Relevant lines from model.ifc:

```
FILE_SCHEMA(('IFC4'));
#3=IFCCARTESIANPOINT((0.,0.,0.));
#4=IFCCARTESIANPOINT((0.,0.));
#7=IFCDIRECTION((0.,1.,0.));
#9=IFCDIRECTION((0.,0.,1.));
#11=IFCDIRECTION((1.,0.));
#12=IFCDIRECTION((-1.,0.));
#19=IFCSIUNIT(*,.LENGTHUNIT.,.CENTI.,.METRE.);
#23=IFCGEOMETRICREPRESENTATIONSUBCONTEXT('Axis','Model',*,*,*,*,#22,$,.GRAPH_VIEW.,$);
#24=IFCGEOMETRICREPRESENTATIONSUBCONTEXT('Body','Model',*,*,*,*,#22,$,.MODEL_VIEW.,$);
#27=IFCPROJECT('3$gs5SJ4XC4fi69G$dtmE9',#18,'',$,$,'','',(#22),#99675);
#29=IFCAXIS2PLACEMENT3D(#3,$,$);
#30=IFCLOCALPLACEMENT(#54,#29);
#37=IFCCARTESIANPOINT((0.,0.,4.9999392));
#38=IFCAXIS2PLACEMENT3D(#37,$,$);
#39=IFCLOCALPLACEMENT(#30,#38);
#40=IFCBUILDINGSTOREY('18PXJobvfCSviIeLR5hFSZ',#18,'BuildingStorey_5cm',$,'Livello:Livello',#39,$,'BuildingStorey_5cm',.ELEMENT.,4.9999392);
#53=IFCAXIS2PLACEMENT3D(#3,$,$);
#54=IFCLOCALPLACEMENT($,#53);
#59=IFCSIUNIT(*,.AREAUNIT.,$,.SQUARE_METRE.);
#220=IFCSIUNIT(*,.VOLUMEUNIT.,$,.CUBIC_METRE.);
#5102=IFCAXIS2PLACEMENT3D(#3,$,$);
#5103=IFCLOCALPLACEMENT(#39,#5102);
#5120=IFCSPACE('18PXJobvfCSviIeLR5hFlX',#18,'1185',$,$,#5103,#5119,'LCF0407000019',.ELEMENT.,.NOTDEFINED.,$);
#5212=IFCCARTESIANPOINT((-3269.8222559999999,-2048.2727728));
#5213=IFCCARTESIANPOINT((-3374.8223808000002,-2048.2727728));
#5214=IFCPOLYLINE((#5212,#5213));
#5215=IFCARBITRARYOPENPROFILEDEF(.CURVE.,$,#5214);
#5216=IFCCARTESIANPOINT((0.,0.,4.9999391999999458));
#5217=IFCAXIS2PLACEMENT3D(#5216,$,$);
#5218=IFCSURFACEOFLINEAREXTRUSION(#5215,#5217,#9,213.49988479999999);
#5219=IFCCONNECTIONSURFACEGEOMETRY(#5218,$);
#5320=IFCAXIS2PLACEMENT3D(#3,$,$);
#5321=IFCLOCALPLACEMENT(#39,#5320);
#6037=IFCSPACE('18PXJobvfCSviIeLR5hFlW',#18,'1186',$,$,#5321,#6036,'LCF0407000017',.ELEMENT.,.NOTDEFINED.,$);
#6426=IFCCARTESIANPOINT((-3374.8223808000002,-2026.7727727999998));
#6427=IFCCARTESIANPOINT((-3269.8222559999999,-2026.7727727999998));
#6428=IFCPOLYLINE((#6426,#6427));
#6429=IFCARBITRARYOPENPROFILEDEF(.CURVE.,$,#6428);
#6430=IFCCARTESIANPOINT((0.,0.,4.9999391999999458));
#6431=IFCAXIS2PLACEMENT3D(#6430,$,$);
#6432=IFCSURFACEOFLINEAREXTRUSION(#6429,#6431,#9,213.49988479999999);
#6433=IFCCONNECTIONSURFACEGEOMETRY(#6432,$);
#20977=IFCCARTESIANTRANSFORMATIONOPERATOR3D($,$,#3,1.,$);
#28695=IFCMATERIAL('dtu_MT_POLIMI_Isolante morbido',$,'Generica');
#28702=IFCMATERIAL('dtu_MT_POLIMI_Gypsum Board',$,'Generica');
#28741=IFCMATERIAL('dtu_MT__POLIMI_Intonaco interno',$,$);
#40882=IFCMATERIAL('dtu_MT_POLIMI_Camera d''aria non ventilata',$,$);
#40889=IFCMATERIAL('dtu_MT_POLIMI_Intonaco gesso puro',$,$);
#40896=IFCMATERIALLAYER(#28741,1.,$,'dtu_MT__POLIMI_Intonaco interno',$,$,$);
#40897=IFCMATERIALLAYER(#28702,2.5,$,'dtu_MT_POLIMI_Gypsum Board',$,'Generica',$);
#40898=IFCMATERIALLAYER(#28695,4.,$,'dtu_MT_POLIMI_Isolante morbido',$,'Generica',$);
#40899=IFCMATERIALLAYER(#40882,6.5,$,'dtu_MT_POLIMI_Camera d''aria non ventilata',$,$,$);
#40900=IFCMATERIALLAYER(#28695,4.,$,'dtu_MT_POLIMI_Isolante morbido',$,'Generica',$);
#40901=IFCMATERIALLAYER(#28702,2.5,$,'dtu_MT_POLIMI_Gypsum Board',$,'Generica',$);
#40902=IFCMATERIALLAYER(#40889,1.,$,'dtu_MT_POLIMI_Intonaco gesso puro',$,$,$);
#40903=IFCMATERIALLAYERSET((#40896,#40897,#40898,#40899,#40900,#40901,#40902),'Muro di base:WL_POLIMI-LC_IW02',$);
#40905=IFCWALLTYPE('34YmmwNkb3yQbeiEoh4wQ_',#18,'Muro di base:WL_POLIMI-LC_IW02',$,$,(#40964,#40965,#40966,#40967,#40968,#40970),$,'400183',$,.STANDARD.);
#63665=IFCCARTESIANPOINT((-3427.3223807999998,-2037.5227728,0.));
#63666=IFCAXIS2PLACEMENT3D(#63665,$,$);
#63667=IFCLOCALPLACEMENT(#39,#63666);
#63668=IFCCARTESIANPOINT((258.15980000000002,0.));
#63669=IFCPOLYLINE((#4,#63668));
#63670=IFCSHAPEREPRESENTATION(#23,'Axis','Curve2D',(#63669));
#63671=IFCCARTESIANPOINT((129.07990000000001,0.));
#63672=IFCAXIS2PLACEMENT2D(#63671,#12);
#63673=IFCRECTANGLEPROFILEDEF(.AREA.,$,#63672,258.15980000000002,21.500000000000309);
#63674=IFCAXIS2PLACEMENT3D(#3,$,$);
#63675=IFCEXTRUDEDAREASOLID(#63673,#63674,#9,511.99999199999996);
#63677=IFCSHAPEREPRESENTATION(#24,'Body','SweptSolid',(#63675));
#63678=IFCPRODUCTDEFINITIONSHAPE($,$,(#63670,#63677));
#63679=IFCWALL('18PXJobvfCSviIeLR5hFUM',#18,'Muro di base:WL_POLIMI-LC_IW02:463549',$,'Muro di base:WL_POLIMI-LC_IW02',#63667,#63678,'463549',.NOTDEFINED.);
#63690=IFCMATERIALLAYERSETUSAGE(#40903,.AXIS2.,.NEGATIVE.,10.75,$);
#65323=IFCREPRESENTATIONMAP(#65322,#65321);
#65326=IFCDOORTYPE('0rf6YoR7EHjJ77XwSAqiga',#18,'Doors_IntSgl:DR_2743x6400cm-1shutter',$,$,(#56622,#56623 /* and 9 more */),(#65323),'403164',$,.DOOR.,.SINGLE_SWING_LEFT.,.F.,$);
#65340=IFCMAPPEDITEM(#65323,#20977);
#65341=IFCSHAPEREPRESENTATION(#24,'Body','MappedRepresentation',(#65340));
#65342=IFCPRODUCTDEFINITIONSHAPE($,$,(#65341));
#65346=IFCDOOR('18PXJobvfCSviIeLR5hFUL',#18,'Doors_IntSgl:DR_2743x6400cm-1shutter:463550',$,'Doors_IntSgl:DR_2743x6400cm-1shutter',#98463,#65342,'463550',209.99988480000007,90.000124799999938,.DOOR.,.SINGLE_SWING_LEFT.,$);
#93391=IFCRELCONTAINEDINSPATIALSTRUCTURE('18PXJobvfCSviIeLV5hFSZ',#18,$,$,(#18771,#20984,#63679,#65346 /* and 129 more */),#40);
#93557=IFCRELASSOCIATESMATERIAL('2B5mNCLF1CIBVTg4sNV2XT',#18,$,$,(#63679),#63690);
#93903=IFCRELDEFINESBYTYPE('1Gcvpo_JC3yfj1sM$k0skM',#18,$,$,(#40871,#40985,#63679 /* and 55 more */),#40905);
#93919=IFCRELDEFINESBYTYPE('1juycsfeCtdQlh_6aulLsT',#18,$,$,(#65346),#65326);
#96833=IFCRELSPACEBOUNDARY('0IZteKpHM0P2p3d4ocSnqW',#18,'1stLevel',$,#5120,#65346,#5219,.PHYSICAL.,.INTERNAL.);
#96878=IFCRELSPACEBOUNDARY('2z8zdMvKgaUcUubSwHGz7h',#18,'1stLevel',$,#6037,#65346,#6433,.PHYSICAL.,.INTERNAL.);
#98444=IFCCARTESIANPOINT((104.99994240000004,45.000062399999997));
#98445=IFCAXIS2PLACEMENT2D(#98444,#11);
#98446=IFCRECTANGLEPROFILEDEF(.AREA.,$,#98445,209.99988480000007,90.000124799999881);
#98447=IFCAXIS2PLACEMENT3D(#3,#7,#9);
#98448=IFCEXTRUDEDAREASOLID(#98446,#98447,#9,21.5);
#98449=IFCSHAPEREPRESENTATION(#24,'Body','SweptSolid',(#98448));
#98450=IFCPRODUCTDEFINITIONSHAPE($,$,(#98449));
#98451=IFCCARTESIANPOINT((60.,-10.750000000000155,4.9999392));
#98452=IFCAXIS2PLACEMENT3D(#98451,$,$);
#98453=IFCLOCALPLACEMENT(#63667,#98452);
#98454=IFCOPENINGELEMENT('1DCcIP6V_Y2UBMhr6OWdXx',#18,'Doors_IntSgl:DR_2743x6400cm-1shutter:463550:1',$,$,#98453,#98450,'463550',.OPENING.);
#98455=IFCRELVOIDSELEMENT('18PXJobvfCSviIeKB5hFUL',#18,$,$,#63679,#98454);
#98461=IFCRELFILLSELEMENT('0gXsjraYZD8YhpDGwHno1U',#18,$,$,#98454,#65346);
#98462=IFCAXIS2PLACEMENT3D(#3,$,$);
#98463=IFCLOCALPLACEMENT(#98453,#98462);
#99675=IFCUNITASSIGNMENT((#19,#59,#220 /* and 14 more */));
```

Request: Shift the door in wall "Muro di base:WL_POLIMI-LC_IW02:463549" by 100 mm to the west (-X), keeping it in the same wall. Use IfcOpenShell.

```python
import numpy as np
import ifcopenshell
import ifcopenshell.api.geometry
import ifcopenshell.util.placement
import ifcopenshell.util.unit

model = ifcopenshell.open("model.ifc")
unit_scale = ifcopenshell.util.unit.calculate_unit_scale(model)

door = model.by_id(65346)
opening = door.FillsVoids[0].RelatingOpeningElement
wall = opening.VoidsElements[0].RelatingBuildingElement

wall_matrix = ifcopenshell.util.placement.get_local_placement(wall.ObjectPlacement)
shift = wall_matrix[:3, 0] * -0.1 / unit_scale
before = ifcopenshell.util.placement.get_local_placement(door.ObjectPlacement)[:3, 3].copy()

# The door is placed relative to its opening, so it follows when the opening moves.
matrix = ifcopenshell.util.placement.get_local_placement(opening.ObjectPlacement)
matrix[:3, 3] += shift
ifcopenshell.api.geometry.edit_object_placement(
    model, product=opening, matrix=matrix, is_si=False, should_transform_children=True
)

# Space boundary surfaces are stored in each space's coordinates; move them too.
for rel in door.ProvidesBoundaries:
    if not rel.ConnectionGeometry:
        continue
    surface = rel.ConnectionGeometry.SurfaceOnRelatingElement
    space_matrix = ifcopenshell.util.placement.get_local_placement(rel.RelatingSpace.ObjectPlacement)
    point = np.array(surface.Position.Location.Coordinates) + space_matrix[:3, :3].T @ shift
    surface.Position = model.createIfcAxis2Placement3D(
        model.createIfcCartesianPoint(point.tolist()), surface.Position.Axis, surface.Position.RefDirection
    )

after = ifcopenshell.util.placement.get_local_placement(door.ObjectPlacement)[:3, 3]
print("door moved by", (after - before).round(3) + 0.0)

model.write("model_v2.ifc")
```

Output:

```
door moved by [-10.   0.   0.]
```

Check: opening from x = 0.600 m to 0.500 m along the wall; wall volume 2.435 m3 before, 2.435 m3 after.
